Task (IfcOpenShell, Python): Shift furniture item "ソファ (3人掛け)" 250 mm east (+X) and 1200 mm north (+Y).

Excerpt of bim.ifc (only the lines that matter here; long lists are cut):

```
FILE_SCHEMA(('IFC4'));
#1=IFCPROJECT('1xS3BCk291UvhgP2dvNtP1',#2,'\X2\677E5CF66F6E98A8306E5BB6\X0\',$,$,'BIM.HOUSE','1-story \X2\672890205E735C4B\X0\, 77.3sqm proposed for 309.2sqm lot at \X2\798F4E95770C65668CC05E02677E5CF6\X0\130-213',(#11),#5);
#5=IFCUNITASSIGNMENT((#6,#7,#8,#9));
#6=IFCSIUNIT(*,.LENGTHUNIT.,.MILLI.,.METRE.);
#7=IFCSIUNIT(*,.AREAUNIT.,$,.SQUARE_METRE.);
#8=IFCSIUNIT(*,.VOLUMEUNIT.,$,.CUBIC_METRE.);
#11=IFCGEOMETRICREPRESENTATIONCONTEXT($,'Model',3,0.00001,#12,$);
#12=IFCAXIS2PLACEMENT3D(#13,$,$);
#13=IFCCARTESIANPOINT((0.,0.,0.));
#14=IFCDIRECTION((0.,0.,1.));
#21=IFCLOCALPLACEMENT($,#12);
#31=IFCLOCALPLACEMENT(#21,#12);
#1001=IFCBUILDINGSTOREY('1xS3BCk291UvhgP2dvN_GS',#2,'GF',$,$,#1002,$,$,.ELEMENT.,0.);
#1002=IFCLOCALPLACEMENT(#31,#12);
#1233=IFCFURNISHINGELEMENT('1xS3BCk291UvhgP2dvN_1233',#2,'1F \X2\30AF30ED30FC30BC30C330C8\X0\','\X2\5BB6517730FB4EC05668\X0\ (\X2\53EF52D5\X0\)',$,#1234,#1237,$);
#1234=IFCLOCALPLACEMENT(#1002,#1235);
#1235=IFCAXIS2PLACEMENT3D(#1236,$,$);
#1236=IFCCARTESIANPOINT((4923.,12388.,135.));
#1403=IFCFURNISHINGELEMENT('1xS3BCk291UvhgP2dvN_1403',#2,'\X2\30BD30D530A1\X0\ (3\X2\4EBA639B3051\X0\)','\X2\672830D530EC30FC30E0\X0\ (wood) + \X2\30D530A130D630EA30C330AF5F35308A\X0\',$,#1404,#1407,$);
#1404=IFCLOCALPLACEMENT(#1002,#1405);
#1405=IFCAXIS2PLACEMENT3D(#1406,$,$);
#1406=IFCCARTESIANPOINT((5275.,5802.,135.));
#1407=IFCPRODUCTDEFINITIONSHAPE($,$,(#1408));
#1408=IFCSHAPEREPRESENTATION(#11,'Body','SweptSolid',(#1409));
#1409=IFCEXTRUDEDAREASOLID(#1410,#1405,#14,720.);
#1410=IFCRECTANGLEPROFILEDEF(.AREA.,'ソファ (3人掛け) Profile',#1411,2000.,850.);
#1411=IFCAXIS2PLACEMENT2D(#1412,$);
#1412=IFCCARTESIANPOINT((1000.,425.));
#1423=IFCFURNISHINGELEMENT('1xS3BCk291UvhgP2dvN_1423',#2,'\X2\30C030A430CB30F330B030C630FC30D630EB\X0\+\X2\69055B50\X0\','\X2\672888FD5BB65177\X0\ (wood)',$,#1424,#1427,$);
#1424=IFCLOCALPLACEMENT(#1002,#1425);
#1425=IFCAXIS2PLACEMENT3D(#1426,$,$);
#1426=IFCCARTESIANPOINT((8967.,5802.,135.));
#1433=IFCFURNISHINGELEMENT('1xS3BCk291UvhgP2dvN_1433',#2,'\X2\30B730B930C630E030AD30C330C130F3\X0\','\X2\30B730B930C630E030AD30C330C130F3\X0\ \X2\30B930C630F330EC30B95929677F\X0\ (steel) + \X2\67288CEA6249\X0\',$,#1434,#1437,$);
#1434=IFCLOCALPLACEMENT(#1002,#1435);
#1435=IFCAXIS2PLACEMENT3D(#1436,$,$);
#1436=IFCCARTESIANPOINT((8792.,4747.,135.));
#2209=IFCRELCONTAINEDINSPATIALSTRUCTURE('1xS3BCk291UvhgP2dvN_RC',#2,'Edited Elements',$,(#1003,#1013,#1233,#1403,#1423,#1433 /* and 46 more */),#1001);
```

```python
import ifcopenshell
import ifcopenshell.api.geometry
import ifcopenshell.util.placement
import ifcopenshell.util.unit

model = ifcopenshell.open("bim.ifc")
unit_scale = ifcopenshell.util.unit.calculate_unit_scale(model)

item = model.by_guid("1xS3BCk291UvhgP2dvN_1403")
matrix = ifcopenshell.util.placement.get_local_placement(item.ObjectPlacement)
matrix[0, 3] += 0.25 / unit_scale
matrix[1, 3] += 1.2 / unit_scale
ifcopenshell.api.geometry.edit_object_placement(model, product=item, matrix=matrix, is_si=False)

print(ifcopenshell.util.placement.get_local_placement(item.ObjectPlacement).round(3) + 0.0)

model.write("bim_rev.ifc")
```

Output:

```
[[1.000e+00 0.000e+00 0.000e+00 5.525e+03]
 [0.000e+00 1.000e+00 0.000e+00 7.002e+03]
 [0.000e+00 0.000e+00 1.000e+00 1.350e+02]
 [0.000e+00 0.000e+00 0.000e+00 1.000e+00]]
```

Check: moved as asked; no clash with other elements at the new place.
